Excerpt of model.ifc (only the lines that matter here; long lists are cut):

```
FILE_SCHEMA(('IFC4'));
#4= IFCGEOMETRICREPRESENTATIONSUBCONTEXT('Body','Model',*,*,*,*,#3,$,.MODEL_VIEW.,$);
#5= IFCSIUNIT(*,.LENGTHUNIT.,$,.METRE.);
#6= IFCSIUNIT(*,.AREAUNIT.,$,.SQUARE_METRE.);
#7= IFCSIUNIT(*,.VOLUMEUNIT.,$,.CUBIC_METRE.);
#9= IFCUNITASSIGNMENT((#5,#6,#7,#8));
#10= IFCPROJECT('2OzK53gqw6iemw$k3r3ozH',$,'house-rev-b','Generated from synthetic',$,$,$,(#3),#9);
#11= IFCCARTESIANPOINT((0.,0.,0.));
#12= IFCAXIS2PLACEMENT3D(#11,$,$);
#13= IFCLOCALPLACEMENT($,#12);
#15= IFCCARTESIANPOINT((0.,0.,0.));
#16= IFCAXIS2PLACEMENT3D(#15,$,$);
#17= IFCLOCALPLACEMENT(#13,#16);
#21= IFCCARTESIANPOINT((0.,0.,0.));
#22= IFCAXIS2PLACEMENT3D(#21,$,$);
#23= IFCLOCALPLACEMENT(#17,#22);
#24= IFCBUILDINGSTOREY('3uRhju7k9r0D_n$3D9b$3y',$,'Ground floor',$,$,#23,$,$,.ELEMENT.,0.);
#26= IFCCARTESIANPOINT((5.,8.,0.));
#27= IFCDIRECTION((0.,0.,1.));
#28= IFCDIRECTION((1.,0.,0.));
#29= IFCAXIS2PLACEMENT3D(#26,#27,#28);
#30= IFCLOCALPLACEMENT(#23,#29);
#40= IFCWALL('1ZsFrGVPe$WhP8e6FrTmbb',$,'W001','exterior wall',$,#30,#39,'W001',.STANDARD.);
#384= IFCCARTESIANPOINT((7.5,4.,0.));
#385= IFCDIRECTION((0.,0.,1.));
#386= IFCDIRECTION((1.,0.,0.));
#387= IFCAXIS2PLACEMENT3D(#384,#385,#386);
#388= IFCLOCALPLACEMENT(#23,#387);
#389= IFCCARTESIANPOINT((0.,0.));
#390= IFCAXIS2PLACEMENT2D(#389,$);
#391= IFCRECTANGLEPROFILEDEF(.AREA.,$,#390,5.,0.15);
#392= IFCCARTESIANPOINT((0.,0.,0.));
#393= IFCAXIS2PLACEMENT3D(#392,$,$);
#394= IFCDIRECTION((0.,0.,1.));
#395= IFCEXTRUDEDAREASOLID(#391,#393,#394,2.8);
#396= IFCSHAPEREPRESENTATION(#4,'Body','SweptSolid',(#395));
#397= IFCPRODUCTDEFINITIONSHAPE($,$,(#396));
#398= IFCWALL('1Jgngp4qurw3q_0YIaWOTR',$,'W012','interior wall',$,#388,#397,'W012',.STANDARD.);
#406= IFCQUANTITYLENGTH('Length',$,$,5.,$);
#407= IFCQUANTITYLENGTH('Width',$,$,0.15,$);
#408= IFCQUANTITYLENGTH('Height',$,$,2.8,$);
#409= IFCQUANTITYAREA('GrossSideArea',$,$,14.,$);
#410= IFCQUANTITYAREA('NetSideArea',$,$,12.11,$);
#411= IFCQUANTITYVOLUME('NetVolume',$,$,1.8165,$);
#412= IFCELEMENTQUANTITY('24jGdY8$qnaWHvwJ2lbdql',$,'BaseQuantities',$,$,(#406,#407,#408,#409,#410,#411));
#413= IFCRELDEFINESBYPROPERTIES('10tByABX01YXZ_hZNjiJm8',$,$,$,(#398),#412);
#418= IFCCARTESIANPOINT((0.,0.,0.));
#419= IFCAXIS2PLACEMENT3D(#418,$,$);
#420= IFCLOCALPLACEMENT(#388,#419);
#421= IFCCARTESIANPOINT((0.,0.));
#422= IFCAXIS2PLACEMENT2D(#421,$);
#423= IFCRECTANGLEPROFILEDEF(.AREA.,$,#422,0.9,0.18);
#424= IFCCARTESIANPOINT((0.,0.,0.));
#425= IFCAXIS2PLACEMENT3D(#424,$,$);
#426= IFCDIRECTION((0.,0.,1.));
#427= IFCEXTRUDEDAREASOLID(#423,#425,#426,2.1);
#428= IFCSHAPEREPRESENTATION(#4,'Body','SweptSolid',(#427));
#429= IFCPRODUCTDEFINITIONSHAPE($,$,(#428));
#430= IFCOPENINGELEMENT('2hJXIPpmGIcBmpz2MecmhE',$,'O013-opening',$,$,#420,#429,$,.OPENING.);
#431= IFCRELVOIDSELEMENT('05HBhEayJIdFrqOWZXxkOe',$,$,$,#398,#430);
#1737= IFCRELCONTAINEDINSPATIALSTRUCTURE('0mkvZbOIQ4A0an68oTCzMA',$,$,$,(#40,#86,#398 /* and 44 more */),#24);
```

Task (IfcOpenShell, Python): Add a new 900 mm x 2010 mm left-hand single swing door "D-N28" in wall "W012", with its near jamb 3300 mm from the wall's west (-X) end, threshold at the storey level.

```python
import numpy as np
import ifcopenshell
import ifcopenshell.api.feature
import ifcopenshell.api.geometry
import ifcopenshell.api.pset
import ifcopenshell.api.root
import ifcopenshell.api.spatial
import ifcopenshell.geom
import ifcopenshell.util.element
import ifcopenshell.util.placement
import ifcopenshell.util.representation
import ifcopenshell.util.shape
import ifcopenshell.util.unit

model = ifcopenshell.open("model.ifc")
unit_scale = ifcopenshell.util.unit.calculate_unit_scale(model)
area_scale = ifcopenshell.util.unit.calculate_unit_scale(model, "AREAUNIT")
volume_scale = ifcopenshell.util.unit.calculate_unit_scale(model, "VOLUMEUNIT")
settings = ifcopenshell.geom.settings()


def volume(element):
    """Net volume in cubic metres, openings subtracted."""
    shape = ifcopenshell.geom.create_shape(settings, element)
    return ifcopenshell.util.shape.get_volume(shape.geometry)


wall = model.by_guid("1Jgngp4qurw3q_0YIaWOTR")
storey = ifcopenshell.util.element.get_container(wall, ifc_class="IfcBuildingStorey")
context = ifcopenshell.util.representation.get_context(model, "Model", "Body", "MODEL_VIEW")
before = volume(wall)

width, height, from_end, sill = 0.9, 2.01, 3.3, 0.0  # metres

# The wall runs along its own X axis, and the end named is its -X end.
wall_shape = ifcopenshell.geom.create_shape(settings, wall)
x, y, z = ifcopenshell.util.shape.get_vertices(wall_shape.geometry).T
start = x.min() + from_end
face, thickness = float(y.min()), float(y.max() - y.min())
wall_matrix = ifcopenshell.util.placement.get_local_placement(wall.ObjectPlacement)
level = ifcopenshell.util.placement.get_local_placement(storey.ObjectPlacement)[2, 3]


def in_wall(x, y):
    """Placement at x, y metres in the wall's axes, at sill height."""
    matrix = wall_matrix.copy()
    matrix[:, 3] = wall_matrix @ np.array([x / unit_scale, y / unit_scale, 0.0, 1.0])
    matrix[2, 3] = level + sill / unit_scale
    return matrix


# Opening: a box that overshoots both wall faces by 50 mm.
opening = ifcopenshell.api.root.create_entity(model, ifc_class="IfcOpeningElement", predefined_type="OPENING")
box = ifcopenshell.api.geometry.add_wall_representation(
    model, context=context, length=width, height=height, thickness=thickness + 0.1
)
ifcopenshell.api.geometry.assign_representation(model, product=opening, representation=box)
ifcopenshell.api.geometry.edit_object_placement(model, product=opening, matrix=in_wall(start, face - 0.05), is_si=False)
ifcopenshell.api.feature.add_feature(model, feature=opening, element=wall)

door = ifcopenshell.api.root.create_entity(model, ifc_class="IfcDoor", name="D-N28", predefined_type="DOOR")
door.OverallWidth, door.OverallHeight = width / unit_scale, height / unit_scale
door.OperationType = "SINGLE_SWING_LEFT"
body = ifcopenshell.api.geometry.add_door_representation(
    model,
    context=context,
    overall_width=door.OverallWidth,
    overall_height=door.OverallHeight,
    operation_type="SINGLE_SWING_LEFT",
    lining_properties={"LiningDepth": thickness / unit_scale, "ThresholdDepth": thickness / unit_scale},
)
ifcopenshell.api.geometry.assign_representation(model, product=door, representation=body)
ifcopenshell.api.spatial.assign_container(model, products=[door], relating_structure=storey)
ifcopenshell.api.feature.add_filling(model, opening=opening, element=door)

# The lining spans the wall, so the door starts at the wall face.
ifcopenshell.api.geometry.edit_object_placement(model, product=door, matrix=in_wall(start, face), is_si=False)

after = volume(wall)

# Update the wall's stored quantities.
qto = model.by_id(ifcopenshell.util.element.get_pset(wall, "BaseQuantities", should_inherit=False)["id"])
ifcopenshell.api.pset.edit_qto(model, qto=qto, properties={
    "NetSideArea": after / thickness / area_scale,
    "NetVolume": after / volume_scale,
})

print(f"wall volume {before:.3f} -> {after:.3f} m3")

model.write("model_rev.ifc")
```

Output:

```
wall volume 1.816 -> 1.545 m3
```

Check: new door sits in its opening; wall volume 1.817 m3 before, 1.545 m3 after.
